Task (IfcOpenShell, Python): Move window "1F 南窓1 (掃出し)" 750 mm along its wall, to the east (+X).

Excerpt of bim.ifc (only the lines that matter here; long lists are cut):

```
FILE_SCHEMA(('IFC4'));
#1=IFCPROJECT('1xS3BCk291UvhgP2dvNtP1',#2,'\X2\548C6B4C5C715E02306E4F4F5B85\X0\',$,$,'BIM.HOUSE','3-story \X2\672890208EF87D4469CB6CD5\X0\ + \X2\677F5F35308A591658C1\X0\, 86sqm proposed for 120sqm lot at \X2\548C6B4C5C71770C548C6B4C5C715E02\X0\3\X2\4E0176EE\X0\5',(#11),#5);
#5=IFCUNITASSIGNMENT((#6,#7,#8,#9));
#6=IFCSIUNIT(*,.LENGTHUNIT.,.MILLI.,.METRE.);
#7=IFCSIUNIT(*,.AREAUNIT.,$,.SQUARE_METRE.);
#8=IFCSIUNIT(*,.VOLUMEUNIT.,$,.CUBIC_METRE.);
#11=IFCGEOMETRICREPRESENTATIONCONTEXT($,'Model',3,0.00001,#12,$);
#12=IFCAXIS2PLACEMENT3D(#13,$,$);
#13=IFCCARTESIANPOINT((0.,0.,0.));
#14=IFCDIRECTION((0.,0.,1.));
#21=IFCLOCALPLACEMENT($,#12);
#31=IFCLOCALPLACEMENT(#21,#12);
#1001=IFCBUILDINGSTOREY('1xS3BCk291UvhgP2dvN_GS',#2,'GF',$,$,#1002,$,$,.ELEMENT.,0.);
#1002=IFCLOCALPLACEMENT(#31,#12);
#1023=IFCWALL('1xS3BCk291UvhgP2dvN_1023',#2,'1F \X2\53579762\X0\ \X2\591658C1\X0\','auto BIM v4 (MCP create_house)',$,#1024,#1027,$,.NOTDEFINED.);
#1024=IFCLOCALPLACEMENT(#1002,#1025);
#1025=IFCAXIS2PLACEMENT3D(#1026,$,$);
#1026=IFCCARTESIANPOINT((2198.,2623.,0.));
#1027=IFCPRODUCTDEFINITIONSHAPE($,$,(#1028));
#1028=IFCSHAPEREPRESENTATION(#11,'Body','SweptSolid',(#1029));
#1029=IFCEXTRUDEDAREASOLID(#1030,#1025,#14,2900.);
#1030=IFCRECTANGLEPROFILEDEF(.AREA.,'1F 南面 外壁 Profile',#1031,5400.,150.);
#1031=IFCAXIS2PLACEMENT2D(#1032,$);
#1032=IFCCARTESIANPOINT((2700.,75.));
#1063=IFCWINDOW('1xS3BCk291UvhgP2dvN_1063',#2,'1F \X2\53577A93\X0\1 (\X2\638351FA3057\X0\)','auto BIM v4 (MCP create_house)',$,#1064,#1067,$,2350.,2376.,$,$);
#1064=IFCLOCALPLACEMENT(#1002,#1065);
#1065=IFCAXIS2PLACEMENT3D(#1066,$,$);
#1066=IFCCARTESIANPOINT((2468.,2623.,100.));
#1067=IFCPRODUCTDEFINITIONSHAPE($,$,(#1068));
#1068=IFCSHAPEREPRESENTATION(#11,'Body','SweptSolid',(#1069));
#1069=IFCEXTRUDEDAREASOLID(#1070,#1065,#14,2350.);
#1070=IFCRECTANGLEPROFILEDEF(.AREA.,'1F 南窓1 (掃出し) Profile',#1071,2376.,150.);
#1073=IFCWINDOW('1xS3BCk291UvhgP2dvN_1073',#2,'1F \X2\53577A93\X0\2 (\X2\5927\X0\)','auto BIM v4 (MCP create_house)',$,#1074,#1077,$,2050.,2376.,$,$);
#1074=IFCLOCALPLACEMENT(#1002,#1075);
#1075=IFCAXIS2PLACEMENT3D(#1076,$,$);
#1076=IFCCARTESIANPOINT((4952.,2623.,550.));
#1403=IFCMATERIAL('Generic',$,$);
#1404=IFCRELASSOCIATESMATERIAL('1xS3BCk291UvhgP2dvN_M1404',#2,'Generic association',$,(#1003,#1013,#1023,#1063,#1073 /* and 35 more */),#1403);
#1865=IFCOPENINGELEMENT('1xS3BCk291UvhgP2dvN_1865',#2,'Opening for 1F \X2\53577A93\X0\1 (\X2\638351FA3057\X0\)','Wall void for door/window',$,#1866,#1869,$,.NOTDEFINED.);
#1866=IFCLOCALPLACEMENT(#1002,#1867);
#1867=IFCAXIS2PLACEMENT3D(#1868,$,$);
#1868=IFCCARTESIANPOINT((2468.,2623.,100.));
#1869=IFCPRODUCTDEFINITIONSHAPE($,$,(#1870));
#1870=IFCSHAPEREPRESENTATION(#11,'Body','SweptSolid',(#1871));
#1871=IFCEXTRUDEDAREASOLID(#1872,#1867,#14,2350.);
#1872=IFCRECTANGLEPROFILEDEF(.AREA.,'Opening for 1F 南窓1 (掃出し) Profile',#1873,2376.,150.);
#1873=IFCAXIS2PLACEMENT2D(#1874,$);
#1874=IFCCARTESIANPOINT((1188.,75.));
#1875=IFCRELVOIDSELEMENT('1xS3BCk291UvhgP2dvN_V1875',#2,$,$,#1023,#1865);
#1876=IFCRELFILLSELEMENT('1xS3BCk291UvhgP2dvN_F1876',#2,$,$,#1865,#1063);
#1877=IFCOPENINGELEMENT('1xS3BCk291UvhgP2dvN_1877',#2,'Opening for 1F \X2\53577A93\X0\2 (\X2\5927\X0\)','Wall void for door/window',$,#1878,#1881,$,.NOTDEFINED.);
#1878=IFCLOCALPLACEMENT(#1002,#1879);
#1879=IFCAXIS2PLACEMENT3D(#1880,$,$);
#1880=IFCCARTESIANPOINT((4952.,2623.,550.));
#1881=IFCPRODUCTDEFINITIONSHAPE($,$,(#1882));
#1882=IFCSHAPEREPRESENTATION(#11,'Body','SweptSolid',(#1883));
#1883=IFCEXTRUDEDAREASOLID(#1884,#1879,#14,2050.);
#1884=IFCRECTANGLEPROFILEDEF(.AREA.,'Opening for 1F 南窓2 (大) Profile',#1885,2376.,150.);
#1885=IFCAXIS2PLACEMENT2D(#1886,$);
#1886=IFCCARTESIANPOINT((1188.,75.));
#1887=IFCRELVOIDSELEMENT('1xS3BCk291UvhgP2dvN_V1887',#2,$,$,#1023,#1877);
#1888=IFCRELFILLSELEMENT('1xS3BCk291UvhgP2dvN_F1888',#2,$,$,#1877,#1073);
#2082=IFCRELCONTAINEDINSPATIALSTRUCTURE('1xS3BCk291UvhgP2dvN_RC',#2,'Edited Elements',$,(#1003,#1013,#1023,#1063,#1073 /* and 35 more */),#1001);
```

```python
import ifcopenshell
import ifcopenshell.api.geometry
import ifcopenshell.util.placement

model = ifcopenshell.open("bim.ifc")

window = model.by_guid("1xS3BCk291UvhgP2dvN_1063")
opening = window.FillsVoids[0].RelatingOpeningElement
wall = opening.VoidsElements[0].RelatingBuildingElement

wall_matrix = ifcopenshell.util.placement.get_local_placement(wall.ObjectPlacement)
shift = wall_matrix[:3, 0] * 750.0
before = ifcopenshell.util.placement.get_local_placement(window.ObjectPlacement)[:3, 3].copy()

# The window is not placed relative to its opening, so move both.
for product in (opening, window):
    matrix = ifcopenshell.util.placement.get_local_placement(product.ObjectPlacement)
    matrix[:3, 3] += shift
    ifcopenshell.api.geometry.edit_object_placement(model, product=product, matrix=matrix, is_si=False)

after = ifcopenshell.util.placement.get_local_placement(window.ObjectPlacement)[:3, 3]
print("window moved by", (after - before).round(3) + 0.0)

model.write("bim_v2.ifc")
```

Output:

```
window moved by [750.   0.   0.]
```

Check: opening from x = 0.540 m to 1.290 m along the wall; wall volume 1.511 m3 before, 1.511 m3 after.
